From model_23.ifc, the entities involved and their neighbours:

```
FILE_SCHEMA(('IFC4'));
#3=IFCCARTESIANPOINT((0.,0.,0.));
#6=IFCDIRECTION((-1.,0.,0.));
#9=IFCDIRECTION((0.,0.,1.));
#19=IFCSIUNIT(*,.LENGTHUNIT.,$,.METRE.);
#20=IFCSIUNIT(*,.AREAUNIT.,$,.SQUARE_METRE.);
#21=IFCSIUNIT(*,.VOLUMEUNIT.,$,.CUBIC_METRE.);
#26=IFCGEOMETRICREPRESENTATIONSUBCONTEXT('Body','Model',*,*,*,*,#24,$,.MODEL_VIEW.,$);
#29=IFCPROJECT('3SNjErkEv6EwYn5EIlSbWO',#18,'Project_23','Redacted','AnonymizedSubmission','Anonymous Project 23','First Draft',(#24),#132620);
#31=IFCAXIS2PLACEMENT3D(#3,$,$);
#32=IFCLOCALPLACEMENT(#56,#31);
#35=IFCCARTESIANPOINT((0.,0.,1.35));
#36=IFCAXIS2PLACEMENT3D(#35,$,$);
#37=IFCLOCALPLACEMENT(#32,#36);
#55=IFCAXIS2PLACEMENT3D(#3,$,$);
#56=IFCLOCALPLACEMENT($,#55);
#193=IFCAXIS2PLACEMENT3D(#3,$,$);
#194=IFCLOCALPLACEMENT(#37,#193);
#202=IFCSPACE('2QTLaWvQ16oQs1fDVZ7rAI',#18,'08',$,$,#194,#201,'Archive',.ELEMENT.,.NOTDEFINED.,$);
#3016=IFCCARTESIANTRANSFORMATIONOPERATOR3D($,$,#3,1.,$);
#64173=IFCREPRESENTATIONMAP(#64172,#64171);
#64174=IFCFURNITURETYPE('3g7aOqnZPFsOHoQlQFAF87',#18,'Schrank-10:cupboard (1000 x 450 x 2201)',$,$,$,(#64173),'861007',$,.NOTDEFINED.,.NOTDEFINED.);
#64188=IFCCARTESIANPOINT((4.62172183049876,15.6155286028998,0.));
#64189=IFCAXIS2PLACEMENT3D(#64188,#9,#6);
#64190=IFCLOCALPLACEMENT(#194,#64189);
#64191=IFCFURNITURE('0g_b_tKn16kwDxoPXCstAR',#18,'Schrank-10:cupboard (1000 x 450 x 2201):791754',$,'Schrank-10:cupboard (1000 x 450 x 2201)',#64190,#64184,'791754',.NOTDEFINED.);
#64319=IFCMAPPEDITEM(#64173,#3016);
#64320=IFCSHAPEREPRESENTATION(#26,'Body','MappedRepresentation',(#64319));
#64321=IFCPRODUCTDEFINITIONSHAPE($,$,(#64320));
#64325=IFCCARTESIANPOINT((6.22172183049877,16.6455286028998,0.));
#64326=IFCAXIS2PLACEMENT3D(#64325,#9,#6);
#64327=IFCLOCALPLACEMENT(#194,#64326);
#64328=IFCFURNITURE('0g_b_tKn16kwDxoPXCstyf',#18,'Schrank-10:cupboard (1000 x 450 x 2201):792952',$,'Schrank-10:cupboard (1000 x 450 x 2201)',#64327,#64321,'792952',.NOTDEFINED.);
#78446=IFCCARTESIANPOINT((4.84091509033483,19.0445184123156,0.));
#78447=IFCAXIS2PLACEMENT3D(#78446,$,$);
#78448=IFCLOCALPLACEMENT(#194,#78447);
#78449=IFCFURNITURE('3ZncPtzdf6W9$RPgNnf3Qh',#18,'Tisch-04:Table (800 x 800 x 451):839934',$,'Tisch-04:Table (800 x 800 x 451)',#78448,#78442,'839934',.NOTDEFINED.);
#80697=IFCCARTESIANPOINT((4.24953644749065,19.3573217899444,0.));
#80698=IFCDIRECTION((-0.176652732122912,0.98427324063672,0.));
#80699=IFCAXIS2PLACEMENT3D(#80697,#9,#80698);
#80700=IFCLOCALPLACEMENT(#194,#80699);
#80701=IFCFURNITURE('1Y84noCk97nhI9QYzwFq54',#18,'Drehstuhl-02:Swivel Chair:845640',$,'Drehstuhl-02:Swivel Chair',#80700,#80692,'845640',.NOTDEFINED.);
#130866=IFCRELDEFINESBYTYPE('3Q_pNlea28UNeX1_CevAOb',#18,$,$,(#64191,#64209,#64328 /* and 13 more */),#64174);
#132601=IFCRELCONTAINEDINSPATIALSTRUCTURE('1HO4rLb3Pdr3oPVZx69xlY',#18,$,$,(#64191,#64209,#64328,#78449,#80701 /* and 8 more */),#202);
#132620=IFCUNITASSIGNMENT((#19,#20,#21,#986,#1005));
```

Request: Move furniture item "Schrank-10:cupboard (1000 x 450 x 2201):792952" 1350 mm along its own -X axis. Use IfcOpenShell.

```python
import ifcopenshell
import ifcopenshell.api.geometry
import ifcopenshell.util.placement

model = ifcopenshell.open("model_23.ifc")

item = model.by_guid("0g_b_tKn16kwDxoPXCstyf")
matrix = ifcopenshell.util.placement.get_local_placement(item.ObjectPlacement)
matrix[:3, 3] -= matrix[:3, 0] * 1.35
ifcopenshell.api.geometry.edit_object_placement(model, product=item, matrix=matrix, is_si=False)

print(ifcopenshell.util.placement.get_local_placement(item.ObjectPlacement).round(3) + 0.0)

model.write("model_23_rev.ifc")
```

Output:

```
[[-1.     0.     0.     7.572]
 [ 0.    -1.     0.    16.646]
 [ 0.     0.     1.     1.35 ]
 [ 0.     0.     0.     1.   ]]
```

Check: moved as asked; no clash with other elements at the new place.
